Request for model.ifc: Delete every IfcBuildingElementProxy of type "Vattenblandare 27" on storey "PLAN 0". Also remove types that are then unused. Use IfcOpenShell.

First a look at what the model holds.

```python
import ifcopenshell
import ifcopenshell.util.element

model = ifcopenshell.open("model.ifc")
print(model.schema)
storey = next(s for s in model.by_type("IfcBuildingStorey") if s.Name == "PLAN 0")
proxies = [e for e in ifcopenshell.util.element.get_decomposition(storey) if e.is_a("IfcBuildingElementProxy")]
seen = {}
for e in proxies:
    element_type = ifcopenshell.util.element.get_type(e)
    name = element_type.Name if element_type not in (None, e) else None
    seen[name] = seen.get(name, 0) + 1
for name, count in sorted(seen.items(), key=str):
    print(count, "x", name)
```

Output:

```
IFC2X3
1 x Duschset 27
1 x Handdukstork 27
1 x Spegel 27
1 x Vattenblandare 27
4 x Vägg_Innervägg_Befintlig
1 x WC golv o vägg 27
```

```python
import ifcopenshell
import ifcopenshell.api.root
import ifcopenshell.util.element

model = ifcopenshell.open("model.ifc")

storey = next(s for s in model.by_type("IfcBuildingStorey") if s.Name == "PLAN 0")
proxies = [e for e in ifcopenshell.util.element.get_decomposition(storey) if e.is_a("IfcBuildingElementProxy")]
targets = [e for e in proxies if (t := ifcopenshell.util.element.get_type(e)) not in (None, e) and t.Name == "Vattenblandare 27"]
types = {ifcopenshell.util.element.get_type(e) for e in targets} - {None, *targets}

for e in targets:
    ifcopenshell.api.root.remove_product(model, product=e)
print(len(targets), "removed")

unused = [t for t in types if not ifcopenshell.util.element.get_types(t)]
for t in unused:
    ifcopenshell.api.root.remove_product(model, product=t)
print(len(unused), "unused types removed")

model.write("model_rev.ifc")
```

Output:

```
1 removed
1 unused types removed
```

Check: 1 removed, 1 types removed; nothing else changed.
